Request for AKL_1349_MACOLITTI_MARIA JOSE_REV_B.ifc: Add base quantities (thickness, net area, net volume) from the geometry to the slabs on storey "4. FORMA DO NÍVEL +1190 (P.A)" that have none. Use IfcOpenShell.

First a look at what the model holds.

```python
import ifcopenshell
import ifcopenshell.util.element
import ifcopenshell.util.unit

model = ifcopenshell.open("AKL_1349_MACOLITTI_MARIA JOSE_REV_B.ifc")
print(model.schema)
for unit_type in ("LENGTHUNIT", "AREAUNIT", "VOLUMEUNIT"):
    print(unit_type, ifcopenshell.util.unit.calculate_unit_scale(model, unit_type))
storey = next(s for s in model.by_type("IfcBuildingStorey") if s.Name == "4. FORMA DO NÍVEL +1190 (P.A)")
slabs = [e for e in ifcopenshell.util.element.get_decomposition(storey) if e.is_a("IfcSlab")]
for e in sorted(slabs, key=lambda e: e.id()):
    print(e.id(), e.is_a(), e.Name, list(ifcopenshell.util.element.get_psets(e, qtos_only=True)), sep=" | ")
```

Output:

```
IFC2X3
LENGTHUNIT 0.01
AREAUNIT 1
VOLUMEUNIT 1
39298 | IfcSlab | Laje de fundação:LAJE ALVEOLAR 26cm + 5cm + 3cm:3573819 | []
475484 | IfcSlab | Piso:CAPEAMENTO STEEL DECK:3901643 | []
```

```python
import ifcopenshell
import ifcopenshell.api.pset
import ifcopenshell.geom
import ifcopenshell.util.element
import ifcopenshell.util.shape
import ifcopenshell.util.unit

model = ifcopenshell.open("AKL_1349_MACOLITTI_MARIA JOSE_REV_B.ifc")
unit_scale = ifcopenshell.util.unit.calculate_unit_scale(model)
area_scale = ifcopenshell.util.unit.calculate_unit_scale(model, "AREAUNIT")
volume_scale = ifcopenshell.util.unit.calculate_unit_scale(model, "VOLUMEUNIT")
settings = ifcopenshell.geom.settings()

storey = next(s for s in model.by_type("IfcBuildingStorey") if s.Name == "4. FORMA DO NÍVEL +1190 (P.A)")
slabs = [e for e in ifcopenshell.util.element.get_decomposition(storey) if e.is_a("IfcSlab")]

for e in sorted(slabs, key=lambda e: e.id()):
    if ifcopenshell.util.element.get_psets(e, qtos_only=True, should_inherit=False):
        continue
    # Geometry comes back in metres, in the element's own axes.
    shape = ifcopenshell.geom.create_shape(settings, e)
    values = {
        "Width": ifcopenshell.util.shape.get_z(shape.geometry) / unit_scale,
        "NetArea": ifcopenshell.util.shape.get_footprint_area(shape.geometry) / area_scale,
        "NetVolume": ifcopenshell.util.shape.get_volume(shape.geometry) / volume_scale,
    }
    qto = ifcopenshell.api.pset.add_qto(model, product=e, name="BaseQuantities")
    ifcopenshell.api.pset.edit_qto(model, qto=qto, properties=values)
    print(e.id(), {k: round(v, 3) for k, v in values.items()})

model.write("AKL_1349_MACOLITTI_MARIA JOSE_REV_B_updated.ifc")
```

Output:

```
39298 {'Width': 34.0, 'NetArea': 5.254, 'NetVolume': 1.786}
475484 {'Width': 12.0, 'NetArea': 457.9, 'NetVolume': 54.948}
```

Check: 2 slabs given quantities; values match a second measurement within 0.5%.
